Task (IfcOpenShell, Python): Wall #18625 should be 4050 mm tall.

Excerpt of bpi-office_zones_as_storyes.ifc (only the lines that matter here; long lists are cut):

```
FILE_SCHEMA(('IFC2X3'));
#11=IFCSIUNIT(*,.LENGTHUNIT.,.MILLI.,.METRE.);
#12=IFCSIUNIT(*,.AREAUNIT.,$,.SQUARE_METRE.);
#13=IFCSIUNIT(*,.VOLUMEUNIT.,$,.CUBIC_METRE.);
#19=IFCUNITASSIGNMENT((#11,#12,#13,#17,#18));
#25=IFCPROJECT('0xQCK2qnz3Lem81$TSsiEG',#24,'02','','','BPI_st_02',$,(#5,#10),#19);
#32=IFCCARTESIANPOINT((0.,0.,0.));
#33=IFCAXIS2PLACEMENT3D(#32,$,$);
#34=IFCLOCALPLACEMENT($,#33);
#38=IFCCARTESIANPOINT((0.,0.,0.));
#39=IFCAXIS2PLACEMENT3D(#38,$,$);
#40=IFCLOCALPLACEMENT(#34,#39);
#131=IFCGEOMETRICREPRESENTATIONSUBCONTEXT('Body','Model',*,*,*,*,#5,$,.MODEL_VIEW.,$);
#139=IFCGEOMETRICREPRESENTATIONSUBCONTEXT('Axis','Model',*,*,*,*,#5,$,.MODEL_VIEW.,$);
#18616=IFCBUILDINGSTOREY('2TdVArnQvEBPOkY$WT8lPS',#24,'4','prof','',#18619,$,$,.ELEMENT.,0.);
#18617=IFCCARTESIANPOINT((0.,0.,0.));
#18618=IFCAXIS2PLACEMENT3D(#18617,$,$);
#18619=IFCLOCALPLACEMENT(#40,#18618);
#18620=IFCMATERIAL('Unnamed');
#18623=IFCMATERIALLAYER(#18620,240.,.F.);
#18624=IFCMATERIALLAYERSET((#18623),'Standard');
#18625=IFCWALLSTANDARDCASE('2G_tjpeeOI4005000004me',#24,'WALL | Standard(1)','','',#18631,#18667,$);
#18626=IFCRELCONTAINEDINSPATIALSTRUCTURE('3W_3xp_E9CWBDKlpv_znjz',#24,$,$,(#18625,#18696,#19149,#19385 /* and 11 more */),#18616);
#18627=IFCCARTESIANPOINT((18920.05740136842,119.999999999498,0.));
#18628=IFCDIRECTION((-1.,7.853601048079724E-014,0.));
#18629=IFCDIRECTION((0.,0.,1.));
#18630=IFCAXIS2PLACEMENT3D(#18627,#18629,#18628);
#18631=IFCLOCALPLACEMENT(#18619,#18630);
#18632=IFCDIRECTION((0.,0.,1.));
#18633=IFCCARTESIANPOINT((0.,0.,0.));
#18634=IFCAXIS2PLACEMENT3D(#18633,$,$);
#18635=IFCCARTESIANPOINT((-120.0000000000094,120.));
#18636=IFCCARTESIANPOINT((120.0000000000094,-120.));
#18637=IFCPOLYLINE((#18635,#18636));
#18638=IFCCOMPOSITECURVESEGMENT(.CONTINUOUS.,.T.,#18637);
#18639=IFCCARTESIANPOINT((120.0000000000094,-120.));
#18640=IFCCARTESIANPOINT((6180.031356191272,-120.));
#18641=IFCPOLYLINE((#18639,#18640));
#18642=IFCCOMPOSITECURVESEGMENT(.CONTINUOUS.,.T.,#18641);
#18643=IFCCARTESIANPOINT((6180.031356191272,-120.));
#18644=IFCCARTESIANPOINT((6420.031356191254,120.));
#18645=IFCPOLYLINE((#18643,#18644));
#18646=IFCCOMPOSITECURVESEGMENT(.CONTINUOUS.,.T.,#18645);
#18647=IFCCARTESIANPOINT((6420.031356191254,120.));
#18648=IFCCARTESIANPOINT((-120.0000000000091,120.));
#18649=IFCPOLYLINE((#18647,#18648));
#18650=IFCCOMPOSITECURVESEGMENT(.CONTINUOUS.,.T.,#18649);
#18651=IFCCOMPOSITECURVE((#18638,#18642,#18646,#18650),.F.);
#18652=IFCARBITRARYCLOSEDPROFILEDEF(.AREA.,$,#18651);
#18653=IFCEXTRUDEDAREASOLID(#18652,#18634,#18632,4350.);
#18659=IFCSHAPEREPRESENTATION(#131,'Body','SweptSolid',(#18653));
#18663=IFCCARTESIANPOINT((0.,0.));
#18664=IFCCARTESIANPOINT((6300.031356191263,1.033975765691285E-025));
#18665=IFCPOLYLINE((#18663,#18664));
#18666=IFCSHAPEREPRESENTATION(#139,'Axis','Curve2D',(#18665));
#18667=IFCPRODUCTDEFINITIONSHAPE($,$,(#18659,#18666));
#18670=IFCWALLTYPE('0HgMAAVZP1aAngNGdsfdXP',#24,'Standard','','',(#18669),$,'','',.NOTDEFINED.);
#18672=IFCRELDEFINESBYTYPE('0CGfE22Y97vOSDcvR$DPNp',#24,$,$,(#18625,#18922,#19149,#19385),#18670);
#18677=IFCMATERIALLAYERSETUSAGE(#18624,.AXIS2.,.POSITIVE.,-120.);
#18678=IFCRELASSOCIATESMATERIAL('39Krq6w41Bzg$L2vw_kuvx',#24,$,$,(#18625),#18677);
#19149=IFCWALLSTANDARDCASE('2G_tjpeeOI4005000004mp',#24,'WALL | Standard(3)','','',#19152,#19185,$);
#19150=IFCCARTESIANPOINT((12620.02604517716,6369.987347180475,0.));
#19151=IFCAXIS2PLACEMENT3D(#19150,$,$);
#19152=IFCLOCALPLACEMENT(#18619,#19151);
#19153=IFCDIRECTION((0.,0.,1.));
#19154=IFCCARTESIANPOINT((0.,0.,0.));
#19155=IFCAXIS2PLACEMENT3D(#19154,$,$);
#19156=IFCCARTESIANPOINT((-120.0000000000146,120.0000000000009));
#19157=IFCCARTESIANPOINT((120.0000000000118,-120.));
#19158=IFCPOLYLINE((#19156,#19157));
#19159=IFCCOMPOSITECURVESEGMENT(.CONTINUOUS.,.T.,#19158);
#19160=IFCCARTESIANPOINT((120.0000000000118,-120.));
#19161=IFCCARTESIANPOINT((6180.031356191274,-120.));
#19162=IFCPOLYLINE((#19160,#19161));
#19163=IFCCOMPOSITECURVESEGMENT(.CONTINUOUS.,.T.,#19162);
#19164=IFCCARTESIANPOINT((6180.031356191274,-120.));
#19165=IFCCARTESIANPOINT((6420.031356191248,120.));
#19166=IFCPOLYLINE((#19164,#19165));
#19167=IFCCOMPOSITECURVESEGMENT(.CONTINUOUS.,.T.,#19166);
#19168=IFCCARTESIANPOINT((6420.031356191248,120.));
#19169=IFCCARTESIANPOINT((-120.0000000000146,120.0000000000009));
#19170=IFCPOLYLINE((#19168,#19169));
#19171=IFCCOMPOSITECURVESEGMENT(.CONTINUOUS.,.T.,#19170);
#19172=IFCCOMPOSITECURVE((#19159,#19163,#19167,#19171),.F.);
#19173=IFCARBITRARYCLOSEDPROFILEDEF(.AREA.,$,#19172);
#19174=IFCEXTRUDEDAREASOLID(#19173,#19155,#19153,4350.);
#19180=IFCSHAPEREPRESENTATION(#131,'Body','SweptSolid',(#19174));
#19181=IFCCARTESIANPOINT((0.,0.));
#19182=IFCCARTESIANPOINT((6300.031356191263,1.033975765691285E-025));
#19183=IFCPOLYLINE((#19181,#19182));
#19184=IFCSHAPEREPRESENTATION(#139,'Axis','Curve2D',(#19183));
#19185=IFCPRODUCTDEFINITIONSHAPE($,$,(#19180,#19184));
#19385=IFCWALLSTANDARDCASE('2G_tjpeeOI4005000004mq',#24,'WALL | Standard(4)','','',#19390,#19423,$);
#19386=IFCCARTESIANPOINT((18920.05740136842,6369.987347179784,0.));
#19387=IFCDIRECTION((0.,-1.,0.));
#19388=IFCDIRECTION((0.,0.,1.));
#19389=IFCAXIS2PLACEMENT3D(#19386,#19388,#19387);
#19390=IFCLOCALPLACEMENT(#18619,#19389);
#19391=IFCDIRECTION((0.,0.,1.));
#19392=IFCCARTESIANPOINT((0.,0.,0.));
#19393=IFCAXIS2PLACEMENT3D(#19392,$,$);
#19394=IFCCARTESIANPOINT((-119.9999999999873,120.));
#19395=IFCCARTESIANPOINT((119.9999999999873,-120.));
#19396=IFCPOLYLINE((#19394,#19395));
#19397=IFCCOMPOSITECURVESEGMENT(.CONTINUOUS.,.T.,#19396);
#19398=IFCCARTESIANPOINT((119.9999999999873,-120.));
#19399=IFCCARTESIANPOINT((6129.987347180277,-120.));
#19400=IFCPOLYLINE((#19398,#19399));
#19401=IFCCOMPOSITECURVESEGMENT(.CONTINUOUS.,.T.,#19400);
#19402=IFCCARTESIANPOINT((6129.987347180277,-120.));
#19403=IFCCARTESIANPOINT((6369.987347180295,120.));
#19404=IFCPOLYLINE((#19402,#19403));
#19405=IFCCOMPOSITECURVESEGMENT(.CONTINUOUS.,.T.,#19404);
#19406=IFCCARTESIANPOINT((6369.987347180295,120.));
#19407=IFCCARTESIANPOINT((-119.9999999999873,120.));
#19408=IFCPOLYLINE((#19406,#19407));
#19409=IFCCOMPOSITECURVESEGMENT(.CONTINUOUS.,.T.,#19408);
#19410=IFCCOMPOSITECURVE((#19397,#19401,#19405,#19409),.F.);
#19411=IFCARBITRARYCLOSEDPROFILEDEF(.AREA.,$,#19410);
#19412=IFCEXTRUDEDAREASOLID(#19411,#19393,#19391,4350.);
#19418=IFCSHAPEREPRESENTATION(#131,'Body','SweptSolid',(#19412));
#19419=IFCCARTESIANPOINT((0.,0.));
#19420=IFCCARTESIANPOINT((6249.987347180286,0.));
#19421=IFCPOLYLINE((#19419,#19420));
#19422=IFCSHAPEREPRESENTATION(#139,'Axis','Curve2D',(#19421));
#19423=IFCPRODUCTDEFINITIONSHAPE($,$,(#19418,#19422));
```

```python
import ifcopenshell
import ifcopenshell.geom
import ifcopenshell.util.representation
import ifcopenshell.util.shape
import ifcopenshell.util.unit

model = ifcopenshell.open("bpi-office_zones_as_storyes.ifc")
unit_scale = ifcopenshell.util.unit.calculate_unit_scale(model)
settings = ifcopenshell.geom.settings()


def volume(element):
    """Net volume in cubic metres, openings subtracted."""
    shape = ifcopenshell.geom.create_shape(settings, element)
    return ifcopenshell.util.shape.get_volume(shape.geometry)


wall = model.by_guid("2G_tjpeeOI4005000004me")
before = volume(wall)

body = ifcopenshell.util.representation.get_representation(wall, "Model", "Body")
solid = body.Items[0]
old_height = solid.Depth
solid.Depth = 4.05 / unit_scale
after = volume(wall)

print(f"height {old_height:g} -> {solid.Depth:g}, volume {before:.3f} -> {after:.3f} m3")

model.write("bpi-office_zones_as_storyes-out.ifc")
```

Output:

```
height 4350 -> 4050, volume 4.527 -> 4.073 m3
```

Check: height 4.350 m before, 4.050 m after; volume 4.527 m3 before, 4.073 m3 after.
